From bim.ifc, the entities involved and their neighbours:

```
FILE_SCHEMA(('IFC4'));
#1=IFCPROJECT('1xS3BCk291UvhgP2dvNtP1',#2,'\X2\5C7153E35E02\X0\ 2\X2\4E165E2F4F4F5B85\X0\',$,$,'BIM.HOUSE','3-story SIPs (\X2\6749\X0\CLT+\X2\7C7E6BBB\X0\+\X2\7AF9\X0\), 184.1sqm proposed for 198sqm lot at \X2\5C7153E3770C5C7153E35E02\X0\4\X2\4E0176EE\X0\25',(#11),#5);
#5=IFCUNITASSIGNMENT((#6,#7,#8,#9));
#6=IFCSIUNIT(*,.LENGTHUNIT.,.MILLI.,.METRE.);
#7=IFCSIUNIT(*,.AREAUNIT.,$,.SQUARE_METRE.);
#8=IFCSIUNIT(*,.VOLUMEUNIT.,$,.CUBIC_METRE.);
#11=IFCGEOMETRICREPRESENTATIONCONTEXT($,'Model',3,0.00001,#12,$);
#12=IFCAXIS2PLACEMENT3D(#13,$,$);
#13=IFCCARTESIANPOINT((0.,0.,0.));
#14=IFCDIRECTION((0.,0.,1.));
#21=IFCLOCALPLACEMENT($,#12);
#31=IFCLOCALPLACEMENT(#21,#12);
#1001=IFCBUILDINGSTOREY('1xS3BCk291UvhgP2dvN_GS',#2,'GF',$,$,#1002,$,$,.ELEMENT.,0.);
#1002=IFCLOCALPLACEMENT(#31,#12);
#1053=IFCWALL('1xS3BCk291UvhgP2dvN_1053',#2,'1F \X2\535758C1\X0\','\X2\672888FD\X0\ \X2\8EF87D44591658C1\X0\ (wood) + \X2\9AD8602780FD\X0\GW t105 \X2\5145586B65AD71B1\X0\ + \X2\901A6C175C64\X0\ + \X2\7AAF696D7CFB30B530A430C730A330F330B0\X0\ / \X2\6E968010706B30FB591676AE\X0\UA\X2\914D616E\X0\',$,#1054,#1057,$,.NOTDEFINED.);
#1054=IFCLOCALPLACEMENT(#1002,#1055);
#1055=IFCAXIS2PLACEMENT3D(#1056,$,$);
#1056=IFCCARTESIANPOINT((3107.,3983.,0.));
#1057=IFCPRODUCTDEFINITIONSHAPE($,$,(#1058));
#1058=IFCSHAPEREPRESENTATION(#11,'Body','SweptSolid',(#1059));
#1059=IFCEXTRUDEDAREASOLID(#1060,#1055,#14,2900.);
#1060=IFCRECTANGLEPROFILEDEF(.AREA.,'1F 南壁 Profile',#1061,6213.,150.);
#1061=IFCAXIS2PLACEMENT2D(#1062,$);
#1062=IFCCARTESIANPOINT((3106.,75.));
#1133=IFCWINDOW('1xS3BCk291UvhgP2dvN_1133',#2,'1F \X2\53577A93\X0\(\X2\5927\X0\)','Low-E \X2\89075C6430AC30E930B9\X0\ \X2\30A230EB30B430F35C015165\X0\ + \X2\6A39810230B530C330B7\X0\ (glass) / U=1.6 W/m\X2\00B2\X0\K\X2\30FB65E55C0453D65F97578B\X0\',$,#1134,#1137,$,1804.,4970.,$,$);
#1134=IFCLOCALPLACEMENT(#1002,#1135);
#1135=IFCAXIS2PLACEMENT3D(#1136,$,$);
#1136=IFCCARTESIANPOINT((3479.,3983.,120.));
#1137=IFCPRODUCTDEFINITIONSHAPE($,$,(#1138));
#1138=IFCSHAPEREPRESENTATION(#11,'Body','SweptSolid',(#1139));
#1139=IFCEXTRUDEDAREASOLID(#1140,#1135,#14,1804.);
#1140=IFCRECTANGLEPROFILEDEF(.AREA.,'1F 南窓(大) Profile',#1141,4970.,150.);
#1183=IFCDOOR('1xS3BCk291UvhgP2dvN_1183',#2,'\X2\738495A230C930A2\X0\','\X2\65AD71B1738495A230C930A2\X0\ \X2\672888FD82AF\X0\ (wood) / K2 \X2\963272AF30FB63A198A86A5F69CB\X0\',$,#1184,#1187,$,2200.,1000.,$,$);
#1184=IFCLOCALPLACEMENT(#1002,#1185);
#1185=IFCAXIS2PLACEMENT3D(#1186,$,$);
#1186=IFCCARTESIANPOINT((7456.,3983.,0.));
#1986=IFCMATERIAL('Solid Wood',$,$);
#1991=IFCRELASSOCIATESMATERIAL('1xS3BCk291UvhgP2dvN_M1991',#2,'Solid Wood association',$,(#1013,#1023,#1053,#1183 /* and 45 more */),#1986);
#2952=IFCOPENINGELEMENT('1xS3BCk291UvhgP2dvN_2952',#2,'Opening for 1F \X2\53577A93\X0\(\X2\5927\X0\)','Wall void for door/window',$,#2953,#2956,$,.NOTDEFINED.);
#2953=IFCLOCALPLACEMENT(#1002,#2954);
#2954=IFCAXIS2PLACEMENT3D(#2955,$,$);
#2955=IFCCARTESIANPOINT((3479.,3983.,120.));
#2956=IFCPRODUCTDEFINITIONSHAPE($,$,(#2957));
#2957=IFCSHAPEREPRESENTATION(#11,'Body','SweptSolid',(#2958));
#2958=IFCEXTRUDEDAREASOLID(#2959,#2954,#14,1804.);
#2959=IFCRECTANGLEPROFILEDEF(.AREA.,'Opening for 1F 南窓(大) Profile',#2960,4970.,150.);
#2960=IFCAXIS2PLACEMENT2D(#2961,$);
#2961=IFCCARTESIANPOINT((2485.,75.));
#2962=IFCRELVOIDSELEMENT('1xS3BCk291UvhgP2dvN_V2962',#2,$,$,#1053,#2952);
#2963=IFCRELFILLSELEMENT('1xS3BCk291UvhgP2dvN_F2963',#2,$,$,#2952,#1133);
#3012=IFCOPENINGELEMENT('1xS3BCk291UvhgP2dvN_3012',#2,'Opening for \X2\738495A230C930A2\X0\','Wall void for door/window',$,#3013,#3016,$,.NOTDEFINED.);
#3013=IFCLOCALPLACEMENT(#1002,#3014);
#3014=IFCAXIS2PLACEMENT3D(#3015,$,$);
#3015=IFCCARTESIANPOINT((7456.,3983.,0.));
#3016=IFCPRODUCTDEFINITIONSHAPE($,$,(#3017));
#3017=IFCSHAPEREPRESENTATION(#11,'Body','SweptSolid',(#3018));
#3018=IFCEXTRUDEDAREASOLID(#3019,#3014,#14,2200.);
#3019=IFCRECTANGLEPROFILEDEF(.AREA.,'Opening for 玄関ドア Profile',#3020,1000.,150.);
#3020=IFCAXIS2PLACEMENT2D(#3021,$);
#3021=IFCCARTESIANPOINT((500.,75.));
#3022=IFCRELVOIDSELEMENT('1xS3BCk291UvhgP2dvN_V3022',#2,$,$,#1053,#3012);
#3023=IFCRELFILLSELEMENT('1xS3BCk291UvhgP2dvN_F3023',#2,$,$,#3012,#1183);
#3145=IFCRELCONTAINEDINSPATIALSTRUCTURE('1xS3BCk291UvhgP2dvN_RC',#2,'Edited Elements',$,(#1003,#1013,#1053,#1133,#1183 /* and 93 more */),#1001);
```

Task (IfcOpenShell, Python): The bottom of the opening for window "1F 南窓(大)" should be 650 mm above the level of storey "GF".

```python
import numpy as np
import ifcopenshell
import ifcopenshell.api.geometry
import ifcopenshell.geom
import ifcopenshell.util.element
import ifcopenshell.util.placement
import ifcopenshell.util.shape
import ifcopenshell.util.unit

model = ifcopenshell.open("bim.ifc")
unit_scale = ifcopenshell.util.unit.calculate_unit_scale(model)

window = model.by_guid("1xS3BCk291UvhgP2dvN_1133")
opening = window.FillsVoids[0].RelatingOpeningElement
storey = ifcopenshell.util.element.get_container(window, ifc_class="IfcBuildingStorey")
level = ifcopenshell.util.placement.get_local_placement(storey.ObjectPlacement)[2, 3]

# The opening's origin need not be at the sill, so measure its lowest point.
shape = ifcopenshell.geom.create_shape(ifcopenshell.geom.settings(), opening)
bottom = ifcopenshell.util.shape.get_shape_bottom_elevation(shape, shape.geometry) / unit_scale
dz = level + 0.65 / unit_scale - bottom

shift = np.array([0.0, 0.0, dz])
# The window is not placed relative to its opening, so move both.
for product in (opening, window):
    matrix = ifcopenshell.util.placement.get_local_placement(product.ObjectPlacement)
    matrix[:3, 3] += shift
    ifcopenshell.api.geometry.edit_object_placement(model, product=product, matrix=matrix, is_si=False)

print(f"moved by {dz * unit_scale:+.3f} m")

model.write("bim_v2.ifc")
```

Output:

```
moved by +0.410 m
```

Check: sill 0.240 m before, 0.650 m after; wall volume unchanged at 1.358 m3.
